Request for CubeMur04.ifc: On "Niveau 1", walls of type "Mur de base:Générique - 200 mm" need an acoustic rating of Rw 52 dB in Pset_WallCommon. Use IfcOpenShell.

First a look at what the model holds.

```python
import ifcopenshell
import ifcopenshell.util.element

model = ifcopenshell.open("CubeMur04.ifc")
print(model.schema)
storey = next(s for s in model.by_type("IfcBuildingStorey") if s.Name == "Niveau 1")
walls = [e for e in ifcopenshell.util.element.get_decomposition(storey) if e.is_a("IfcWall")]
seen = {}
for e in walls:
    element_type = ifcopenshell.util.element.get_type(e)
    key = (element_type.Name if element_type != e and element_type else None, ifcopenshell.util.element.get_pset(e, "Pset_WallCommon", "AcousticRating"))
    seen[key] = seen.get(key, 0) + 1
for (name, value), count in sorted(seen.items(), key=str):
    print(count, "x", name, "|", value)
```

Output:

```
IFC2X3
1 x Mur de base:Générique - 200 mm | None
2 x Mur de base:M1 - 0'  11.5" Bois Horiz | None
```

```python
import ifcopenshell
import ifcopenshell.api.pset
import ifcopenshell.util.element

model = ifcopenshell.open("CubeMur04.ifc")

storey = next(s for s in model.by_type("IfcBuildingStorey") if s.Name == "Niveau 1")
walls = [e for e in ifcopenshell.util.element.get_decomposition(storey) if e.is_a("IfcWall")]

count = 0
for e in walls:
    element_type = ifcopenshell.util.element.get_type(e)
    if element_type in (None, e) or element_type.Name != "Mur de base:Générique - 200 mm":
        continue
    # add_pset returns the element's existing set when there is one.
    pset = ifcopenshell.api.pset.add_pset(model, product=e, name="Pset_WallCommon")
    ifcopenshell.api.pset.edit_pset(model, pset=pset, properties={"AcousticRating": "Rw 52 dB"})
    count += 1

print(count, "walls updated")

model.write("CubeMur04_updated.ifc")
```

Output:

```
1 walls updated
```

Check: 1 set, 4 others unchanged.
